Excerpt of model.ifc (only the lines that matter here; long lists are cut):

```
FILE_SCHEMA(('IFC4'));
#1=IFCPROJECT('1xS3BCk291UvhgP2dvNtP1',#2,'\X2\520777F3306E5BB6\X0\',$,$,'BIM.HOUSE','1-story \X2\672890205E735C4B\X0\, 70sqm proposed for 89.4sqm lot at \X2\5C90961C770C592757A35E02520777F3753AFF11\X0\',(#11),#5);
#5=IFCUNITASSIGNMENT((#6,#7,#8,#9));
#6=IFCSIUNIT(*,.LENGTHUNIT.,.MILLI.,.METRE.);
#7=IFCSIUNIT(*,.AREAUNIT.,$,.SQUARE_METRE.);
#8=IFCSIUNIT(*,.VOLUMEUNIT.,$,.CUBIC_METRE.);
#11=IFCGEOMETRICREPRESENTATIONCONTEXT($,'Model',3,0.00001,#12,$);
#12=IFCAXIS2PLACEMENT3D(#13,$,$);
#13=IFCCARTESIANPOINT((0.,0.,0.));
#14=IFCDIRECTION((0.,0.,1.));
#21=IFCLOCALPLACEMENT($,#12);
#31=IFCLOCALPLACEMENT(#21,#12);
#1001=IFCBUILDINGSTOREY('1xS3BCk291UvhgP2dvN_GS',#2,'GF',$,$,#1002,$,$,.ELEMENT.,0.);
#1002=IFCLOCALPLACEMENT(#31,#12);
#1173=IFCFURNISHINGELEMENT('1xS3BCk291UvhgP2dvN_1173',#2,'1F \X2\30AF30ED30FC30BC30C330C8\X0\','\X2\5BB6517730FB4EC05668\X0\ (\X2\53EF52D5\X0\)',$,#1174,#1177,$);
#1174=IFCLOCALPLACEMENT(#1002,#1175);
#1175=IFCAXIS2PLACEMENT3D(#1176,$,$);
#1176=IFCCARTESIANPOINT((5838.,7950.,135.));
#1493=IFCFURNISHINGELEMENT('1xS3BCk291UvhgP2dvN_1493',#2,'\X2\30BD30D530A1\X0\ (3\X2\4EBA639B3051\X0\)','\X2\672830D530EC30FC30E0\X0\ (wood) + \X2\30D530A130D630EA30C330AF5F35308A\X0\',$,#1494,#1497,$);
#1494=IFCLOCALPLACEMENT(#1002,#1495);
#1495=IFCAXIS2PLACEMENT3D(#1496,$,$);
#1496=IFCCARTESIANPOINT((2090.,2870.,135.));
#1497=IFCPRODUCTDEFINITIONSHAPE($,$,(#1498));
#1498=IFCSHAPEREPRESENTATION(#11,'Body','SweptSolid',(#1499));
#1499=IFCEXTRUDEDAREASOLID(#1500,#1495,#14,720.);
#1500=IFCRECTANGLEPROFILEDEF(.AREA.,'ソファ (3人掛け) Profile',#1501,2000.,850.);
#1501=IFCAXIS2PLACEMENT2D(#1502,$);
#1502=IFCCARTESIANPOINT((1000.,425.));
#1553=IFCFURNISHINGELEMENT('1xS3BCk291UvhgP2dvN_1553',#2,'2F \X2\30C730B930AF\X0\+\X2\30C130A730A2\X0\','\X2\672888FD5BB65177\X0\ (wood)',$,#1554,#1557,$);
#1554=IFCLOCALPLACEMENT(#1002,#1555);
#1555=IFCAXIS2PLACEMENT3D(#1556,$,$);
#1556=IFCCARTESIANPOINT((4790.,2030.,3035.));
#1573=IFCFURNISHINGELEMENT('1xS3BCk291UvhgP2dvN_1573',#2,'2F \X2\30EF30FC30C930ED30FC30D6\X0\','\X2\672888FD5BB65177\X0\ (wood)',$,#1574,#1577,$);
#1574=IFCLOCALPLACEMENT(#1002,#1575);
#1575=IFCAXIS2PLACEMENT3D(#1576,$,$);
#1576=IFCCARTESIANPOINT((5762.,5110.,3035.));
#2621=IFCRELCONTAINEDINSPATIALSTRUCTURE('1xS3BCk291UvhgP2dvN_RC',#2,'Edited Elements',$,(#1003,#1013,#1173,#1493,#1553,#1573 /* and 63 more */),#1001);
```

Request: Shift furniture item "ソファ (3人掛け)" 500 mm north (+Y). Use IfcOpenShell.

```python
import ifcopenshell
import ifcopenshell.api.geometry
import ifcopenshell.util.placement

model = ifcopenshell.open("model.ifc")

item = model.by_guid("1xS3BCk291UvhgP2dvN_1493")
matrix = ifcopenshell.util.placement.get_local_placement(item.ObjectPlacement)
matrix[1, 3] += 500.0
ifcopenshell.api.geometry.edit_object_placement(model, product=item, matrix=matrix, is_si=False)

print(ifcopenshell.util.placement.get_local_placement(item.ObjectPlacement).round(3) + 0.0)

model.write("model_edited.ifc")
```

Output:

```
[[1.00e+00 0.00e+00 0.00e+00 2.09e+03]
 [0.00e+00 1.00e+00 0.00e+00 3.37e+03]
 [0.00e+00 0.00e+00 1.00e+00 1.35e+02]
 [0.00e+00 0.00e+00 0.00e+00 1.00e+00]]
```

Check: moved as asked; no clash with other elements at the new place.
